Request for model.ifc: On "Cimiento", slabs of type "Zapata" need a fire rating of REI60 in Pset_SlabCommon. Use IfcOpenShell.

First a look at what the model holds.

```python
import ifcopenshell
import ifcopenshell.util.element

model = ifcopenshell.open("model.ifc")
print(model.schema)
storey = next(s for s in model.by_type("IfcBuildingStorey") if s.Name == "Cimiento")
slabs = [e for e in ifcopenshell.util.element.get_decomposition(storey) if e.is_a("IfcSlab")]
seen = {}
for e in slabs:
    element_type = ifcopenshell.util.element.get_type(e)
    key = (element_type.Name if element_type != e and element_type else None, ifcopenshell.util.element.get_pset(e, "Pset_SlabCommon", "FireRating"))
    seen[key] = seen.get(key, 0) + 1
for (name, value), count in sorted(seen.items(), key=str):
    print(count, "x", name, "|", value)
```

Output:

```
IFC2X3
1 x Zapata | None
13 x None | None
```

```python
import ifcopenshell
import ifcopenshell.api.pset
import ifcopenshell.util.element

model = ifcopenshell.open("model.ifc")

storey = next(s for s in model.by_type("IfcBuildingStorey") if s.Name == "Cimiento")
slabs = [e for e in ifcopenshell.util.element.get_decomposition(storey) if e.is_a("IfcSlab")]

count = 0
for e in slabs:
    element_type = ifcopenshell.util.element.get_type(e)
    if element_type in (None, e) or element_type.Name != "Zapata":
        continue
    # add_pset returns the element's existing set when there is one.
    pset = ifcopenshell.api.pset.add_pset(model, product=e, name="Pset_SlabCommon")
    ifcopenshell.api.pset.edit_pset(model, pset=pset, properties={"FireRating": "REI60"})
    count += 1

print(count, "slabs updated")

model.write("model_v2.ifc")
```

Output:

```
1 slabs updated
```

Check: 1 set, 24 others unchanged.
